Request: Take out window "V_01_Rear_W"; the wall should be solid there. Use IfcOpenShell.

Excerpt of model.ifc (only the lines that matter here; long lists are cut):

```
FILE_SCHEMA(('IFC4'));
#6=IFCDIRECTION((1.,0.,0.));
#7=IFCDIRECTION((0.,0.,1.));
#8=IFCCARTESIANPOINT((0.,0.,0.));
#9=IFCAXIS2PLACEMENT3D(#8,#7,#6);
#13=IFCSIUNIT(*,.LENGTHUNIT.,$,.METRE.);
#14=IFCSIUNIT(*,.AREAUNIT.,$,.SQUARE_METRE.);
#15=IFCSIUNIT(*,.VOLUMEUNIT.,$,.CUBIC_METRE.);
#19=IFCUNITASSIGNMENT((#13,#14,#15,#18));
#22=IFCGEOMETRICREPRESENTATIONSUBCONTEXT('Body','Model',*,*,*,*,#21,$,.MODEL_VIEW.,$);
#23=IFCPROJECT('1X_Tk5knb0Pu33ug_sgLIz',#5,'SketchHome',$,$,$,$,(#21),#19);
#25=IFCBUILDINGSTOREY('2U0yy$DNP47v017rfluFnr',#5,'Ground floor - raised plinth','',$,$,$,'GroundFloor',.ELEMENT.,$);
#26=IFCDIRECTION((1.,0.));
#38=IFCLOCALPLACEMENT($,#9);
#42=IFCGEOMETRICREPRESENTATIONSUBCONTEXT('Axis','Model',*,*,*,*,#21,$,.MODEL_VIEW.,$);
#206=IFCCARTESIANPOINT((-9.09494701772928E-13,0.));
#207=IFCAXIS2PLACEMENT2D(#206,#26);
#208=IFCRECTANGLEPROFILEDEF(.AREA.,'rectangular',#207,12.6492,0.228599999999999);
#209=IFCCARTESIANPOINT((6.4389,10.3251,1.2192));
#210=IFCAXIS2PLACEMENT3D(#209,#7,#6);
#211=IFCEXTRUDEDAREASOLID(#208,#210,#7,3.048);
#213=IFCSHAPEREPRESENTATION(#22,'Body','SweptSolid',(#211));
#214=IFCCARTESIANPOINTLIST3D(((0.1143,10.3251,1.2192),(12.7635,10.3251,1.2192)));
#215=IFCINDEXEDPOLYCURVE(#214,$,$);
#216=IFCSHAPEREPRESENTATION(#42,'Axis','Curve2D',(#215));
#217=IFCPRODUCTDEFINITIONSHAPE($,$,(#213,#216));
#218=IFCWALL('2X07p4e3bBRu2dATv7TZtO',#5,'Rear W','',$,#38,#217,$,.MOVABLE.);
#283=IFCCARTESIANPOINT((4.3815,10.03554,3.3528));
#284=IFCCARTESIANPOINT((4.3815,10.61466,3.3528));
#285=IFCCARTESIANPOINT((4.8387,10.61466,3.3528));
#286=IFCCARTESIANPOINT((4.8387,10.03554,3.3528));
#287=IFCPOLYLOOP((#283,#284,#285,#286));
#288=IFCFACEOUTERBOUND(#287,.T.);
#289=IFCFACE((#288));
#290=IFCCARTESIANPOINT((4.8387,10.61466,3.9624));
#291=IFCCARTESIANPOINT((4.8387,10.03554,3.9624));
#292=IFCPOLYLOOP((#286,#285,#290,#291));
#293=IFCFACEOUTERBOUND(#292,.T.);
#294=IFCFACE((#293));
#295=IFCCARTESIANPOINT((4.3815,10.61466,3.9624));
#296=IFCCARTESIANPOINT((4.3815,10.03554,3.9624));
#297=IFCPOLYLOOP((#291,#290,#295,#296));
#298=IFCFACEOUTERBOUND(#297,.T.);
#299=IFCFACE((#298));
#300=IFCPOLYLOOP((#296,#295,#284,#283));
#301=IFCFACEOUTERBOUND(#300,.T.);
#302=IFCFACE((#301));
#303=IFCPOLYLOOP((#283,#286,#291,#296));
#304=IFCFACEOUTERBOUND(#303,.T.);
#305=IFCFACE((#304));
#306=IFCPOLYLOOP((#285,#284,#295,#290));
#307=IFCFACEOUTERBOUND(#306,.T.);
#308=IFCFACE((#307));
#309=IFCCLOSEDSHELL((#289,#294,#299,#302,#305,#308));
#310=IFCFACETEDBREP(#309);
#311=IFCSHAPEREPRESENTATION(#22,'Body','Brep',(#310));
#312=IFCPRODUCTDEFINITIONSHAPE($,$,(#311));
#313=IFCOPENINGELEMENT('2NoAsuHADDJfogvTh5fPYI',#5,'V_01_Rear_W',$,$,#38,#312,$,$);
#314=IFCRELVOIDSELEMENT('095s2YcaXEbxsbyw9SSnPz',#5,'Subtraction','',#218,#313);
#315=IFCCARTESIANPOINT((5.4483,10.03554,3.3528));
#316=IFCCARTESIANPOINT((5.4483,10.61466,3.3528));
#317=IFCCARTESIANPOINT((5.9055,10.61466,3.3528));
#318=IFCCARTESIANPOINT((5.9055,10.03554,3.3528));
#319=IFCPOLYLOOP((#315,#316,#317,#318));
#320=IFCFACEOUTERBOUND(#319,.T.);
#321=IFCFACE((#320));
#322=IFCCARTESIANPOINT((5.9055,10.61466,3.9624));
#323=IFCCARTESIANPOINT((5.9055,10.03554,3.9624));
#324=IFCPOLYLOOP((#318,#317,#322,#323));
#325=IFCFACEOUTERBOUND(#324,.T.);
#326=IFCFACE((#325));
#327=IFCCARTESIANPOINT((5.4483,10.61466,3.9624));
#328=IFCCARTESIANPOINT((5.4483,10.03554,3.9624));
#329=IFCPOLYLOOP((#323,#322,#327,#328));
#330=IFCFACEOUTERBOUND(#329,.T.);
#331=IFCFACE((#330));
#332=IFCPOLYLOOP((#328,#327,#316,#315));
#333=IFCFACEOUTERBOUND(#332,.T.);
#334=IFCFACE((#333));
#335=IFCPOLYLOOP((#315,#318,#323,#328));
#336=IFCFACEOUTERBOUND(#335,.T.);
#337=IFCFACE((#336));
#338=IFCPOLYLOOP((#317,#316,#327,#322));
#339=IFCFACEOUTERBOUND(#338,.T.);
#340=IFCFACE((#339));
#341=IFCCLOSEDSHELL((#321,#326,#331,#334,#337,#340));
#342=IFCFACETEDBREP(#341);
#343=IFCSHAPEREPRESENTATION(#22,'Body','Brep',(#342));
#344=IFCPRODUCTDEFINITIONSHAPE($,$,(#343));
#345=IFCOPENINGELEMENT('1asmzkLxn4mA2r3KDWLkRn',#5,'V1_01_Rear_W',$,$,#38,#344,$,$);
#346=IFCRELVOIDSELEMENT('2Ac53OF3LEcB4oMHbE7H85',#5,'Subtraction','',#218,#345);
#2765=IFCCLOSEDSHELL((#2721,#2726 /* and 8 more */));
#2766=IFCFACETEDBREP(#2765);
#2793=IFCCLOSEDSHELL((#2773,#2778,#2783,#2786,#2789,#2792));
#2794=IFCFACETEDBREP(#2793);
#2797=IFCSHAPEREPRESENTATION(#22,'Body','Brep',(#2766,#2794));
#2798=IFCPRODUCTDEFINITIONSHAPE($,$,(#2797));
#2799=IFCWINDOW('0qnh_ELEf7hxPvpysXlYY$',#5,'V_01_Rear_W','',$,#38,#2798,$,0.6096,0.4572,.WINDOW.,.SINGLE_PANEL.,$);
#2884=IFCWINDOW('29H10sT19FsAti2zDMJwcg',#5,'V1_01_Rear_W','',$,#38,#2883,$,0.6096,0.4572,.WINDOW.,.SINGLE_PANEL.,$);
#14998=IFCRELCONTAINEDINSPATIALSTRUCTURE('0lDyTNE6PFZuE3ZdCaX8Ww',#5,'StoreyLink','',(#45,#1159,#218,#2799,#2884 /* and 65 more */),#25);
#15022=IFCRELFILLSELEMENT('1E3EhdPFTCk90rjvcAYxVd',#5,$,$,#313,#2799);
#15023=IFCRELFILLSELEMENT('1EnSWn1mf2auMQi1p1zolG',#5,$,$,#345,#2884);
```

```python
import ifcopenshell
import ifcopenshell.api.feature
import ifcopenshell.api.root
import ifcopenshell.geom
import ifcopenshell.util.shape

model = ifcopenshell.open("model.ifc")
settings = ifcopenshell.geom.settings()


def volume(element):
    """Net volume in cubic metres, openings subtracted."""
    shape = ifcopenshell.geom.create_shape(settings, element)
    return ifcopenshell.util.shape.get_volume(shape.geometry)


window = model.by_guid("0qnh_ELEf7hxPvpysXlYY$")
opening = window.FillsVoids[0].RelatingOpeningElement
wall = opening.VoidsElements[0].RelatingBuildingElement
before = volume(wall)

ifcopenshell.api.root.remove_product(model, product=window)
ifcopenshell.api.feature.remove_feature(model, feature=opening)

after = volume(wall)

print(f"wall volume {before:.3f} -> {after:.3f} m3")

model.write("model_rev.ifc")
```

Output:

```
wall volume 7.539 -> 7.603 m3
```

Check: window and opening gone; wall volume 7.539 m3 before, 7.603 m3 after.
